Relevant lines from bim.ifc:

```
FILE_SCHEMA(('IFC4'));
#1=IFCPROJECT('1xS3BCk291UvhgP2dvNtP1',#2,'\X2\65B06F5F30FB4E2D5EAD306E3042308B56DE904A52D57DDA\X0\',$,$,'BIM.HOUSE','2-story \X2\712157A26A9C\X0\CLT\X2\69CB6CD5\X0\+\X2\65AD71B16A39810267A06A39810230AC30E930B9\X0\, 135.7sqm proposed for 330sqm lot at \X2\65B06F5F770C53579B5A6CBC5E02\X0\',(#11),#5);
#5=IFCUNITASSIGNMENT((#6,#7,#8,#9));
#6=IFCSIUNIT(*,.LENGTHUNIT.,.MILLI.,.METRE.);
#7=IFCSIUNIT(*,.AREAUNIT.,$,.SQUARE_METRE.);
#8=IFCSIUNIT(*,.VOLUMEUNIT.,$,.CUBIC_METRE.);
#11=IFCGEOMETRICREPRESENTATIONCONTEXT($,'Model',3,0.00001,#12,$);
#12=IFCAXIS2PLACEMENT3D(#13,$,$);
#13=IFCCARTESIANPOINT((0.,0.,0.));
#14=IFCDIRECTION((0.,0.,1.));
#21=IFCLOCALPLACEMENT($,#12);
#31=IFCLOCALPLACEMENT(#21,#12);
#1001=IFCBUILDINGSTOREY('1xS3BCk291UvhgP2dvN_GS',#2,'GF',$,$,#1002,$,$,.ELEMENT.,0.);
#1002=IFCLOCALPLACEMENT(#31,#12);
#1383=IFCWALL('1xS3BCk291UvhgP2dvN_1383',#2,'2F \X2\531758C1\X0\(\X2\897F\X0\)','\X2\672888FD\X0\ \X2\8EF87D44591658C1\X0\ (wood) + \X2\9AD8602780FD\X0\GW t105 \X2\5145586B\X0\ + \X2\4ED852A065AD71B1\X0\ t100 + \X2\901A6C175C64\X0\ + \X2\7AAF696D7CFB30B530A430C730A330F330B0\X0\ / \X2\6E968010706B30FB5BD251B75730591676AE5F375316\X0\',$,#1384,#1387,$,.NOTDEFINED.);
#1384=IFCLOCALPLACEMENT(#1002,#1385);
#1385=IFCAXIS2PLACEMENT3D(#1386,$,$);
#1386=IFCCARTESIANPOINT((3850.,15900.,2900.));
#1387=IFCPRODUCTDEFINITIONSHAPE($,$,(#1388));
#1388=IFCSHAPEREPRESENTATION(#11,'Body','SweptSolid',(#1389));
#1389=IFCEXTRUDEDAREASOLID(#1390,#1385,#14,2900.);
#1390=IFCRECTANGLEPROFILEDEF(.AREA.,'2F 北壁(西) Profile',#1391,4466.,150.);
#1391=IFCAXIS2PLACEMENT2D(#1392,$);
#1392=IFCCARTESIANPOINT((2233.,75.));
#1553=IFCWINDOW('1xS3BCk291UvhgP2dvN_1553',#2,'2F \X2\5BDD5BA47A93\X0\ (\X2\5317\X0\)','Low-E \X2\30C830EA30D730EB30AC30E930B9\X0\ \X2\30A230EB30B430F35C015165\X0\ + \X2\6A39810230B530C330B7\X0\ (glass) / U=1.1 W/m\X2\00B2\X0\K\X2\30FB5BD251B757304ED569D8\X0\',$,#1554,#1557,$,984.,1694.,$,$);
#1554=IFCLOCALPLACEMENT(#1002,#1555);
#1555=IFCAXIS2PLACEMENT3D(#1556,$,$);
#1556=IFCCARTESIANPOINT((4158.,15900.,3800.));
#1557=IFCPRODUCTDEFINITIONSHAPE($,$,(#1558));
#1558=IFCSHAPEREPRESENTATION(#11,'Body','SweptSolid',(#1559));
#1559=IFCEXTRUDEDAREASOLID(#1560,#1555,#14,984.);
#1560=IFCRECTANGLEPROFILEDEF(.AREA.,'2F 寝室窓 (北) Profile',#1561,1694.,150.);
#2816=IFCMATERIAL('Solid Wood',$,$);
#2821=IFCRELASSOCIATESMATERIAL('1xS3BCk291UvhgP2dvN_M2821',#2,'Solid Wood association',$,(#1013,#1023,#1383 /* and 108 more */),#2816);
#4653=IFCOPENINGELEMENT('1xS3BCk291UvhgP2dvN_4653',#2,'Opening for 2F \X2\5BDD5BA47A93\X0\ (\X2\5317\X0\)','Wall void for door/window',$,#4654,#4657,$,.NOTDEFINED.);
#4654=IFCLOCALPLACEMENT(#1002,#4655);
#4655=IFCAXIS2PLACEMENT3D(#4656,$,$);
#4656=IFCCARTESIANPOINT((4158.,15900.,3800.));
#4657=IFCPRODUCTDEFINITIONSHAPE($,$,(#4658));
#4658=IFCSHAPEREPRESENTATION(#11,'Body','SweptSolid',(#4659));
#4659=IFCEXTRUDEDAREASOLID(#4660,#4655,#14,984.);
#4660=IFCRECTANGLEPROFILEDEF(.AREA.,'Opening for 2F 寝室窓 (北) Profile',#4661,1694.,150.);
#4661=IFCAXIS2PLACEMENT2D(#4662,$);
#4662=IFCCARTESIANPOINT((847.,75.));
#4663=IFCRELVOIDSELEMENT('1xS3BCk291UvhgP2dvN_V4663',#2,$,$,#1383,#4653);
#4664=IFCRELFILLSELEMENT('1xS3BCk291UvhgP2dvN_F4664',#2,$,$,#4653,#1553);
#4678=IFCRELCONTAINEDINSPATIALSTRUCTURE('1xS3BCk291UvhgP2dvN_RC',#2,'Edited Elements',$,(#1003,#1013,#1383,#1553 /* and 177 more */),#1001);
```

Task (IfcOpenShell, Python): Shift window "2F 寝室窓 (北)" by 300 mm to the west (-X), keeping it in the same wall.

```python
import ifcopenshell
import ifcopenshell.api.geometry
import ifcopenshell.util.placement
import ifcopenshell.util.unit

model = ifcopenshell.open("bim.ifc")
unit_scale = ifcopenshell.util.unit.calculate_unit_scale(model)

window = model.by_id(1553)
opening = window.FillsVoids[0].RelatingOpeningElement
wall = opening.VoidsElements[0].RelatingBuildingElement

wall_matrix = ifcopenshell.util.placement.get_local_placement(wall.ObjectPlacement)
shift = wall_matrix[:3, 0] * -0.3 / unit_scale
before = ifcopenshell.util.placement.get_local_placement(window.ObjectPlacement)[:3, 3].copy()

# The window is not placed relative to its opening, so move both.
for product in (opening, window):
    matrix = ifcopenshell.util.placement.get_local_placement(product.ObjectPlacement)
    matrix[:3, 3] += shift
    ifcopenshell.api.geometry.edit_object_placement(model, product=product, matrix=matrix, is_si=False)

after = ifcopenshell.util.placement.get_local_placement(window.ObjectPlacement)[:3, 3]
print("window moved by", (after - before).round(3) + 0.0)

model.write("bim_edited.ifc")
```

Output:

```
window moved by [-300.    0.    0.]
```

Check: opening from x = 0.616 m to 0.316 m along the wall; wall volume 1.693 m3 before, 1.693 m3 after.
